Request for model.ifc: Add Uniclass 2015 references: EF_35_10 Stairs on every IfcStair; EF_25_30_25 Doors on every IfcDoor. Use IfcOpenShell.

First a look at what the model holds.

```python
import ifcopenshell

model = ifcopenshell.open("model.ifc")
print(model.schema)
print("classifications:", [c.Name for c in model.by_type("IfcClassification")])
for ifc_class in ("IfcDoor", "IfcRoof", "IfcStair", "IfcWall", "IfcWindow"):
    print(ifc_class, len(model.by_type(ifc_class)))
```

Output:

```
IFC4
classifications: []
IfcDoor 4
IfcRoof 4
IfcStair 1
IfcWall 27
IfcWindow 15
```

```python
import ifcopenshell
import ifcopenshell.api.classification

model = ifcopenshell.open("model.ifc")

system = ifcopenshell.api.classification.add_classification(model, classification="Uniclass 2015")

codes = {
    "IfcStair": ("EF_35_10", "Stairs"),
    "IfcDoor": ("EF_25_30_25", "Doors"),
}
for ifc_class, (code, name) in codes.items():
    products = model.by_type(ifc_class)
    ifcopenshell.api.classification.add_reference(
        model, products=products, classification=system, identification=code, name=name
    )
    print(code, len(products))

model.write("model-out.ifc")
```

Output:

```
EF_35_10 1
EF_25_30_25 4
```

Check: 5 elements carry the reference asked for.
